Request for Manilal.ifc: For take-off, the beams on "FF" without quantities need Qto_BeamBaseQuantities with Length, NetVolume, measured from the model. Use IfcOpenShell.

First a look at what the model holds.

```python
import ifcopenshell
import ifcopenshell.util.element
import ifcopenshell.util.unit

model = ifcopenshell.open("Manilal.ifc")
print(model.schema)
for unit_type in ("LENGTHUNIT", "AREAUNIT", "VOLUMEUNIT"):
    print(unit_type, ifcopenshell.util.unit.calculate_unit_scale(model, unit_type))
storey = next(s for s in model.by_type("IfcBuildingStorey") if s.Name == "FF")
beams = [e for e in ifcopenshell.util.element.get_decomposition(storey) if e.is_a("IfcBeam")]
for e in sorted(beams, key=lambda e: e.id()):
    print(e.id(), e.is_a(), e.Name, list(ifcopenshell.util.element.get_psets(e, qtos_only=True)), sep=" | ")
```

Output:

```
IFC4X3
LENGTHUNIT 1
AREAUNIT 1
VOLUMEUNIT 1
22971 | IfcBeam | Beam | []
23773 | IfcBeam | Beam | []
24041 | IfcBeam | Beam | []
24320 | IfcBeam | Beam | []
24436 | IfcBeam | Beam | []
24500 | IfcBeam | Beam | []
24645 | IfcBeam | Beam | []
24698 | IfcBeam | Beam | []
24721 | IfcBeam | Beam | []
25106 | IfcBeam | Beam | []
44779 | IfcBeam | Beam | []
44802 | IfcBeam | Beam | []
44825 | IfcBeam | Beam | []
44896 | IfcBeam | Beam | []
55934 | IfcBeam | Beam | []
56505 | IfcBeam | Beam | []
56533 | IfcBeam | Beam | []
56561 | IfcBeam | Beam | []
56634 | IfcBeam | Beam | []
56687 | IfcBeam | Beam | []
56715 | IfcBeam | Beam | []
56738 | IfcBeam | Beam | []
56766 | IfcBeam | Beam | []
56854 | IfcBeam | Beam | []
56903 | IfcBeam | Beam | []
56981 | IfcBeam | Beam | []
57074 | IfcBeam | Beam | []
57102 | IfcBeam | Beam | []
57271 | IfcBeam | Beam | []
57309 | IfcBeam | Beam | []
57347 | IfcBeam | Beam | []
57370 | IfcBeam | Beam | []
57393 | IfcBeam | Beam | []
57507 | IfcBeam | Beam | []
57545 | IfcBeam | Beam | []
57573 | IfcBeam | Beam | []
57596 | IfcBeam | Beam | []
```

```python
import ifcopenshell
import ifcopenshell.api.pset
import ifcopenshell.geom
import ifcopenshell.util.element
import ifcopenshell.util.shape
import ifcopenshell.util.unit

model = ifcopenshell.open("Manilal.ifc")
unit_scale = ifcopenshell.util.unit.calculate_unit_scale(model)
volume_scale = ifcopenshell.util.unit.calculate_unit_scale(model, "VOLUMEUNIT")
settings = ifcopenshell.geom.settings()

storey = next(s for s in model.by_type("IfcBuildingStorey") if s.Name == "FF")
beams = [e for e in ifcopenshell.util.element.get_decomposition(storey) if e.is_a("IfcBeam")]

for e in sorted(beams, key=lambda e: e.id()):
    if ifcopenshell.util.element.get_psets(e, qtos_only=True, should_inherit=False):
        continue
    # Geometry comes back in metres, in the element's own axes.
    shape = ifcopenshell.geom.create_shape(settings, e)
    values = {
        "Length": ifcopenshell.util.shape.get_max_xyz(shape.geometry) / unit_scale,
        "NetVolume": ifcopenshell.util.shape.get_volume(shape.geometry) / volume_scale,
    }
    qto = ifcopenshell.api.pset.add_qto(model, product=e, name="Qto_BeamBaseQuantities")
    ifcopenshell.api.pset.edit_qto(model, qto=qto, properties=values)
    print(e.id(), {k: round(v, 3) for k, v in values.items()})

model.write("Manilal_edited.ifc")
```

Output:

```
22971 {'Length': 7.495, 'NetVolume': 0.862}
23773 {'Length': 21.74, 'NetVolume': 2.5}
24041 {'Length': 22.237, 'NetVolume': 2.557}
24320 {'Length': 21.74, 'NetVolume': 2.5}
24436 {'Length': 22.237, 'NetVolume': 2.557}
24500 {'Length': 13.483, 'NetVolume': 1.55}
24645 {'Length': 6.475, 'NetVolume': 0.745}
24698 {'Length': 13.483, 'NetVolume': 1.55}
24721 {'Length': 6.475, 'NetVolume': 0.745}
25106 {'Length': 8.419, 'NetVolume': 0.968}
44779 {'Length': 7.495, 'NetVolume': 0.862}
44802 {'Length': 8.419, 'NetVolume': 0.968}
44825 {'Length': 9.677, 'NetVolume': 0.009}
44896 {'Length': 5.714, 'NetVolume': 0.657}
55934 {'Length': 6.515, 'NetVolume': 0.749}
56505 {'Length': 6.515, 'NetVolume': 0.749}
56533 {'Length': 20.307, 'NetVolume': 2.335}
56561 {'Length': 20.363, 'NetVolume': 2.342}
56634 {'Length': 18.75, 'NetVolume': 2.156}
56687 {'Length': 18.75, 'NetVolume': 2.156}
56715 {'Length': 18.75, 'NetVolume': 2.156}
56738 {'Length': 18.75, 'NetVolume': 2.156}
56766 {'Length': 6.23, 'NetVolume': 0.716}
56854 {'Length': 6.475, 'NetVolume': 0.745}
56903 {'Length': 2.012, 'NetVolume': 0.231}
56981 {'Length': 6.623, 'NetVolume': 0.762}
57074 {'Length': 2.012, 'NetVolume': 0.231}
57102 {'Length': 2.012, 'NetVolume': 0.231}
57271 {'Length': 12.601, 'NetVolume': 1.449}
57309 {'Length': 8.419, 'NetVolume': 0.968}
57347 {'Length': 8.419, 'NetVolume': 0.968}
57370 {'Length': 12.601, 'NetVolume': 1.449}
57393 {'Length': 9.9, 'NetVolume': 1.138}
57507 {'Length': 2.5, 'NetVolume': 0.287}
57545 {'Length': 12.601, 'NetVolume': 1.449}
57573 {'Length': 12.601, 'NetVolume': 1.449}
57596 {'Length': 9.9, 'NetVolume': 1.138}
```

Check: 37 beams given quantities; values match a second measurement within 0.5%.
